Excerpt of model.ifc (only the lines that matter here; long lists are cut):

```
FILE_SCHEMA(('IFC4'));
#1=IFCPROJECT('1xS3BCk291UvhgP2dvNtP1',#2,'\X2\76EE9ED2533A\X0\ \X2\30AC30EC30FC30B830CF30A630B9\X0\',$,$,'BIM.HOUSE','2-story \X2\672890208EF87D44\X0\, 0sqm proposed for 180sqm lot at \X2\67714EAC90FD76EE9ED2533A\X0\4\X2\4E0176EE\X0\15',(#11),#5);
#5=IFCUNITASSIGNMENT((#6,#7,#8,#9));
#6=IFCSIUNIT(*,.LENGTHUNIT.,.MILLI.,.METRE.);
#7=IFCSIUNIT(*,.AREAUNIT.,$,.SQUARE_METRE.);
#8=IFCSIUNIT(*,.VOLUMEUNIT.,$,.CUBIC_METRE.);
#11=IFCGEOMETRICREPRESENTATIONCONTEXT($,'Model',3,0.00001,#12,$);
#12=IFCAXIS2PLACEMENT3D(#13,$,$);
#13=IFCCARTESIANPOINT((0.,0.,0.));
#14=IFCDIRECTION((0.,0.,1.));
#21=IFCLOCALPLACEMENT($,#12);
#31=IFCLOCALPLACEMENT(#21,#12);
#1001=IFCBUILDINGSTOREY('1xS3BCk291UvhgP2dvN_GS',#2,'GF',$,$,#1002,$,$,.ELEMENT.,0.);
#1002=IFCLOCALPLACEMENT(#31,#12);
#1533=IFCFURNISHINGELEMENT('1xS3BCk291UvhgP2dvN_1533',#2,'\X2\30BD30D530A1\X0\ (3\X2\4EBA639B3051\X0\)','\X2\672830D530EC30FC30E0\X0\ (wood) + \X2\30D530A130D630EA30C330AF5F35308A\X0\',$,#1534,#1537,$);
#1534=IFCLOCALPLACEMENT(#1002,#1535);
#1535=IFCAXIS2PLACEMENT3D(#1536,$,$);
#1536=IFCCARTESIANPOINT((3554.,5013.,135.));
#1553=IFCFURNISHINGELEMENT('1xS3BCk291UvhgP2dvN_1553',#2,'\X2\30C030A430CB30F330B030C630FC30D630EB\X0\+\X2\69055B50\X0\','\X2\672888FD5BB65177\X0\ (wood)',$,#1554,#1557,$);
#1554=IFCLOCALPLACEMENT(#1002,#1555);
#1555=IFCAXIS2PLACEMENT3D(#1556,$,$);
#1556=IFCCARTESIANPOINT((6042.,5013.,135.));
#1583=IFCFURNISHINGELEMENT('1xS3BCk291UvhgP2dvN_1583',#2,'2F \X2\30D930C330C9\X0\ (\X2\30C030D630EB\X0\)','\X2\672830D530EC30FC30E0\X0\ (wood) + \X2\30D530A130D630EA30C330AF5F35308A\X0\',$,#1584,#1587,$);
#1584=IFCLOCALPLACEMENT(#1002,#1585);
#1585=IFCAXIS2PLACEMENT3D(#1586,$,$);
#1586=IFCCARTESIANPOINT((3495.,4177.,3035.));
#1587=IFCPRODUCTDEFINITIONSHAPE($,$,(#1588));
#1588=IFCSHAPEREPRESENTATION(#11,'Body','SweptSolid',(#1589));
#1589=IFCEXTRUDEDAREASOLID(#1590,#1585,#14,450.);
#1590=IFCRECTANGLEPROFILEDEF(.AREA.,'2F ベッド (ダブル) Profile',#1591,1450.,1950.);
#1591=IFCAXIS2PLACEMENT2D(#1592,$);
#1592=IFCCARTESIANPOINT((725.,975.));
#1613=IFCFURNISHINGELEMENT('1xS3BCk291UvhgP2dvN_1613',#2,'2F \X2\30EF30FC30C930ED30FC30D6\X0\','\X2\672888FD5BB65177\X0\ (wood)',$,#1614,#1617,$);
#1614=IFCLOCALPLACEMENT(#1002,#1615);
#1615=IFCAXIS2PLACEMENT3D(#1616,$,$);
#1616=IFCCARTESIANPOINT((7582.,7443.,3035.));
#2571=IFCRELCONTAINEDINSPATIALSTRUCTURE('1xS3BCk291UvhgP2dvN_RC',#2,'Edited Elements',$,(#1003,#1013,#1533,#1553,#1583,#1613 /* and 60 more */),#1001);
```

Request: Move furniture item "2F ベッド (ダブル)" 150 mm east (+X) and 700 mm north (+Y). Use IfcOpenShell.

```python
import ifcopenshell
import ifcopenshell.api.geometry
import ifcopenshell.util.placement

model = ifcopenshell.open("model.ifc")

item = model.by_guid("1xS3BCk291UvhgP2dvN_1583")
matrix = ifcopenshell.util.placement.get_local_placement(item.ObjectPlacement)
matrix[0, 3] += 150.0
matrix[1, 3] += 700.0
ifcopenshell.api.geometry.edit_object_placement(model, product=item, matrix=matrix, is_si=False)

print(ifcopenshell.util.placement.get_local_placement(item.ObjectPlacement).round(3) + 0.0)

model.write("model_rev.ifc")
```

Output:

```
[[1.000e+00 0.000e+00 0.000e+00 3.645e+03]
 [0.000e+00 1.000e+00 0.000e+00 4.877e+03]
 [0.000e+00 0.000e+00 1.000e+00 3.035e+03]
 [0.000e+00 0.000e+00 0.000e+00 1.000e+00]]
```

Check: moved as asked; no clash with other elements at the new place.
